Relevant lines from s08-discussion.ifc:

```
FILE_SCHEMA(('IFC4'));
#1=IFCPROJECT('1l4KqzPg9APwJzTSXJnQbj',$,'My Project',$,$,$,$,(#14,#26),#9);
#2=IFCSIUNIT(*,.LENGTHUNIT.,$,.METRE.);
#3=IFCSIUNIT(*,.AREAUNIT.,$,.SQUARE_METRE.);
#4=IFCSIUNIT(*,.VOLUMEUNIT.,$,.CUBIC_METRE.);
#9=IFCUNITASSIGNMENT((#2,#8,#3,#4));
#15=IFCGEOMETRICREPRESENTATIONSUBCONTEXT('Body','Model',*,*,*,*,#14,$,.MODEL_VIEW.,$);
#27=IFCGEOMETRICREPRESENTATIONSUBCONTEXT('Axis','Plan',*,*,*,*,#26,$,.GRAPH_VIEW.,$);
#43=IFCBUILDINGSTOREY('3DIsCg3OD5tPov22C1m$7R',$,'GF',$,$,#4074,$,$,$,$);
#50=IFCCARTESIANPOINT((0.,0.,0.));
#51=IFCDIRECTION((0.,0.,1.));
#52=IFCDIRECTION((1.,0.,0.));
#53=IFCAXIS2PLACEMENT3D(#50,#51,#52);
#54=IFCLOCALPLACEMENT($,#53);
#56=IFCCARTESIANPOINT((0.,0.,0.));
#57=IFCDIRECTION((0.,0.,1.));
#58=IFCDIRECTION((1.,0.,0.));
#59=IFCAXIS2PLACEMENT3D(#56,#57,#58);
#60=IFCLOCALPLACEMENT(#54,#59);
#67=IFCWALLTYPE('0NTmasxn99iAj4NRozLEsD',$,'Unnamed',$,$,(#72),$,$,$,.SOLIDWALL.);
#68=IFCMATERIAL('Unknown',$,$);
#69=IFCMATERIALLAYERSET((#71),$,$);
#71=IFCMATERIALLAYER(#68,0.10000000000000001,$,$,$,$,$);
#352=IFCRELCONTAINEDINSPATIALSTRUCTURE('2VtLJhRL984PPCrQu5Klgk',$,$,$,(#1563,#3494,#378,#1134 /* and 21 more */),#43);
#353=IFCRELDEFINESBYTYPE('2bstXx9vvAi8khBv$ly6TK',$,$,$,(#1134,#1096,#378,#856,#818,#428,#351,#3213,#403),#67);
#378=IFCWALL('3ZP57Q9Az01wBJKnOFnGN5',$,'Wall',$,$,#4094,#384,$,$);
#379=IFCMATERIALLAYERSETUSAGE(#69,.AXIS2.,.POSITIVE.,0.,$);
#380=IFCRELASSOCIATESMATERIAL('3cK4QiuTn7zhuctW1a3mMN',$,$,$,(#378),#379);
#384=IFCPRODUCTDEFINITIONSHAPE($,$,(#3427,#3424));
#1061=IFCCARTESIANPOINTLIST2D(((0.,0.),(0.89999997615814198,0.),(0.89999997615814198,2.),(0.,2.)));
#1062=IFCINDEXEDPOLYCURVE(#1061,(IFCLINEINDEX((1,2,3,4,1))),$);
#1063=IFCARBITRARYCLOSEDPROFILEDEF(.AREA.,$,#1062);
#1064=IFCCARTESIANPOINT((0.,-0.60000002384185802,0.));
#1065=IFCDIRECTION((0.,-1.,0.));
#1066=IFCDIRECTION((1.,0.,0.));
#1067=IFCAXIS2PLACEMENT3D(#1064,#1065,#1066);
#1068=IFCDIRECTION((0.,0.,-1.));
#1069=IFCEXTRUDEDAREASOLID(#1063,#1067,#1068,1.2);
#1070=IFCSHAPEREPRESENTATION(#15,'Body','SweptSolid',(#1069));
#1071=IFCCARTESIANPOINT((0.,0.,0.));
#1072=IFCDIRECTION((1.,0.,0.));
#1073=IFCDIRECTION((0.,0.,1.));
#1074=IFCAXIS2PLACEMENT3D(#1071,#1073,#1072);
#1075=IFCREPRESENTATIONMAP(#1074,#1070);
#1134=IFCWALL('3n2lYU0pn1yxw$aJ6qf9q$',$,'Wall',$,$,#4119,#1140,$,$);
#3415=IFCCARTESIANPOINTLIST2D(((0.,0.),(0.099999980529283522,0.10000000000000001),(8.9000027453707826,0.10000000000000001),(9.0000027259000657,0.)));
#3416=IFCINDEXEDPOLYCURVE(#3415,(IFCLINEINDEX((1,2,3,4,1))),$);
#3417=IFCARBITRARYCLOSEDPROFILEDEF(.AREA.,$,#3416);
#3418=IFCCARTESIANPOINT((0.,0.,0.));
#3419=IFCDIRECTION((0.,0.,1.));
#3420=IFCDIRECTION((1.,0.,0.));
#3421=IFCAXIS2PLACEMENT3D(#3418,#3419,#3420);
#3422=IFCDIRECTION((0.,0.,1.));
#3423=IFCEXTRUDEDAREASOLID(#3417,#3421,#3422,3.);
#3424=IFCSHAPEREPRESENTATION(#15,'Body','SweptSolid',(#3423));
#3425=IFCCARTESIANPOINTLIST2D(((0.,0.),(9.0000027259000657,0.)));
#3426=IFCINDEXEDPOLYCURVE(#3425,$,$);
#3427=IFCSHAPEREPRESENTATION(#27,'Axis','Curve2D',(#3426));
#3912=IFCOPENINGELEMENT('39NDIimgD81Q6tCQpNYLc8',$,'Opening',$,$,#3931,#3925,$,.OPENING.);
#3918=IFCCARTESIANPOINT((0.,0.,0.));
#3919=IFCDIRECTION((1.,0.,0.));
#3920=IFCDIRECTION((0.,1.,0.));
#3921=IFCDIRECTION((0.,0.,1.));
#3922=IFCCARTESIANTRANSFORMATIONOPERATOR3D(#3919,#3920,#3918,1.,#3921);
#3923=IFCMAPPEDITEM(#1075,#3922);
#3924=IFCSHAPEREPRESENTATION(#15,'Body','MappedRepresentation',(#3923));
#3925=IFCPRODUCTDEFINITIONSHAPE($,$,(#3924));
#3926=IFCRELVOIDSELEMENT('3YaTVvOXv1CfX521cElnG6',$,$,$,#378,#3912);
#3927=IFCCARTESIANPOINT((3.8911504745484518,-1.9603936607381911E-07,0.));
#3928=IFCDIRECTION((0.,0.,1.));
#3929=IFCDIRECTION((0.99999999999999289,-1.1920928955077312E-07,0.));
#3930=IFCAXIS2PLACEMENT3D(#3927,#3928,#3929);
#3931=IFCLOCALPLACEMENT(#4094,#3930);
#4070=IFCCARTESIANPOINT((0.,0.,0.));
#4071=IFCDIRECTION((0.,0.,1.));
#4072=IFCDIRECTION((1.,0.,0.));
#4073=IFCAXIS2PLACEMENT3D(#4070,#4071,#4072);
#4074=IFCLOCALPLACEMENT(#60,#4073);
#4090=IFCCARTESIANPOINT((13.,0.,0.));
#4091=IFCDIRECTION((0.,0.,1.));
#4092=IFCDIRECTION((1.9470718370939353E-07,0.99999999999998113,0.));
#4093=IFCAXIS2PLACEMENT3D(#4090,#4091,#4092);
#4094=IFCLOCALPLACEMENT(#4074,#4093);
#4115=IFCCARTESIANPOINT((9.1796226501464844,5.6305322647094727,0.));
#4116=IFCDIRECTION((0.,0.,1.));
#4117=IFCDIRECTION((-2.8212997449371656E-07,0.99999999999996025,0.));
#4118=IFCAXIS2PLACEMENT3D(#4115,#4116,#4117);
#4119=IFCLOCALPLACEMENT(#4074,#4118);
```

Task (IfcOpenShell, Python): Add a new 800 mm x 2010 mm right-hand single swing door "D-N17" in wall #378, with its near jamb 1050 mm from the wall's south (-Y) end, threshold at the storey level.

```python
import numpy as np
import ifcopenshell
import ifcopenshell.api.feature
import ifcopenshell.api.geometry
import ifcopenshell.api.root
import ifcopenshell.api.spatial
import ifcopenshell.geom
import ifcopenshell.util.element
import ifcopenshell.util.placement
import ifcopenshell.util.representation
import ifcopenshell.util.shape
import ifcopenshell.util.unit

model = ifcopenshell.open("s08-discussion.ifc")
unit_scale = ifcopenshell.util.unit.calculate_unit_scale(model)
settings = ifcopenshell.geom.settings()


def volume(element):
    """Net volume in cubic metres, openings subtracted."""
    shape = ifcopenshell.geom.create_shape(settings, element)
    return ifcopenshell.util.shape.get_volume(shape.geometry)


wall = model.by_guid("3ZP57Q9Az01wBJKnOFnGN5")
storey = ifcopenshell.util.element.get_container(wall, ifc_class="IfcBuildingStorey")
context = ifcopenshell.util.representation.get_context(model, "Model", "Body", "MODEL_VIEW")
before = volume(wall)

width, height, from_end, sill = 0.8, 2.01, 1.05, 0.0  # metres

# The wall runs along its own X axis, and the end named is its -X end.
wall_shape = ifcopenshell.geom.create_shape(settings, wall)
x, y, z = ifcopenshell.util.shape.get_vertices(wall_shape.geometry).T
start = x.min() + from_end
face, thickness = float(y.min()), float(y.max() - y.min())
wall_matrix = ifcopenshell.util.placement.get_local_placement(wall.ObjectPlacement)
level = ifcopenshell.util.placement.get_local_placement(storey.ObjectPlacement)[2, 3]


def in_wall(x, y):
    """Placement at x, y metres in the wall's axes, at sill height."""
    matrix = wall_matrix.copy()
    matrix[:, 3] = wall_matrix @ np.array([x / unit_scale, y / unit_scale, 0.0, 1.0])
    matrix[2, 3] = level + sill / unit_scale
    return matrix


# Opening: a box that overshoots both wall faces by 50 mm.
opening = ifcopenshell.api.root.create_entity(model, ifc_class="IfcOpeningElement", predefined_type="OPENING")
box = ifcopenshell.api.geometry.add_wall_representation(
    model, context=context, length=width, height=height, thickness=thickness + 0.1
)
ifcopenshell.api.geometry.assign_representation(model, product=opening, representation=box)
ifcopenshell.api.geometry.edit_object_placement(model, product=opening, matrix=in_wall(start, face - 0.05), is_si=False)
ifcopenshell.api.feature.add_feature(model, feature=opening, element=wall)

door = ifcopenshell.api.root.create_entity(model, ifc_class="IfcDoor", name="D-N17", predefined_type="DOOR")
door.OverallWidth, door.OverallHeight = width / unit_scale, height / unit_scale
door.OperationType = "SINGLE_SWING_RIGHT"
body = ifcopenshell.api.geometry.add_door_representation(
    model,
    context=context,
    overall_width=door.OverallWidth,
    overall_height=door.OverallHeight,
    operation_type="SINGLE_SWING_RIGHT",
    lining_properties={"LiningDepth": thickness / unit_scale, "ThresholdDepth": thickness / unit_scale},
)
ifcopenshell.api.geometry.assign_representation(model, product=door, representation=body)
ifcopenshell.api.spatial.assign_container(model, products=[door], relating_structure=storey)
ifcopenshell.api.feature.add_filling(model, opening=opening, element=door)

# The lining spans the wall, so the door starts at the wall face.
ifcopenshell.api.geometry.edit_object_placement(model, product=door, matrix=in_wall(start, face), is_si=False)

after = volume(wall)

print(f"wall volume {before:.3f} -> {after:.3f} m3")

model.write("s08-discussion-out.ifc")
```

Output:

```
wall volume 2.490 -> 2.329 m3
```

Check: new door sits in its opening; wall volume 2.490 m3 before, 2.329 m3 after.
